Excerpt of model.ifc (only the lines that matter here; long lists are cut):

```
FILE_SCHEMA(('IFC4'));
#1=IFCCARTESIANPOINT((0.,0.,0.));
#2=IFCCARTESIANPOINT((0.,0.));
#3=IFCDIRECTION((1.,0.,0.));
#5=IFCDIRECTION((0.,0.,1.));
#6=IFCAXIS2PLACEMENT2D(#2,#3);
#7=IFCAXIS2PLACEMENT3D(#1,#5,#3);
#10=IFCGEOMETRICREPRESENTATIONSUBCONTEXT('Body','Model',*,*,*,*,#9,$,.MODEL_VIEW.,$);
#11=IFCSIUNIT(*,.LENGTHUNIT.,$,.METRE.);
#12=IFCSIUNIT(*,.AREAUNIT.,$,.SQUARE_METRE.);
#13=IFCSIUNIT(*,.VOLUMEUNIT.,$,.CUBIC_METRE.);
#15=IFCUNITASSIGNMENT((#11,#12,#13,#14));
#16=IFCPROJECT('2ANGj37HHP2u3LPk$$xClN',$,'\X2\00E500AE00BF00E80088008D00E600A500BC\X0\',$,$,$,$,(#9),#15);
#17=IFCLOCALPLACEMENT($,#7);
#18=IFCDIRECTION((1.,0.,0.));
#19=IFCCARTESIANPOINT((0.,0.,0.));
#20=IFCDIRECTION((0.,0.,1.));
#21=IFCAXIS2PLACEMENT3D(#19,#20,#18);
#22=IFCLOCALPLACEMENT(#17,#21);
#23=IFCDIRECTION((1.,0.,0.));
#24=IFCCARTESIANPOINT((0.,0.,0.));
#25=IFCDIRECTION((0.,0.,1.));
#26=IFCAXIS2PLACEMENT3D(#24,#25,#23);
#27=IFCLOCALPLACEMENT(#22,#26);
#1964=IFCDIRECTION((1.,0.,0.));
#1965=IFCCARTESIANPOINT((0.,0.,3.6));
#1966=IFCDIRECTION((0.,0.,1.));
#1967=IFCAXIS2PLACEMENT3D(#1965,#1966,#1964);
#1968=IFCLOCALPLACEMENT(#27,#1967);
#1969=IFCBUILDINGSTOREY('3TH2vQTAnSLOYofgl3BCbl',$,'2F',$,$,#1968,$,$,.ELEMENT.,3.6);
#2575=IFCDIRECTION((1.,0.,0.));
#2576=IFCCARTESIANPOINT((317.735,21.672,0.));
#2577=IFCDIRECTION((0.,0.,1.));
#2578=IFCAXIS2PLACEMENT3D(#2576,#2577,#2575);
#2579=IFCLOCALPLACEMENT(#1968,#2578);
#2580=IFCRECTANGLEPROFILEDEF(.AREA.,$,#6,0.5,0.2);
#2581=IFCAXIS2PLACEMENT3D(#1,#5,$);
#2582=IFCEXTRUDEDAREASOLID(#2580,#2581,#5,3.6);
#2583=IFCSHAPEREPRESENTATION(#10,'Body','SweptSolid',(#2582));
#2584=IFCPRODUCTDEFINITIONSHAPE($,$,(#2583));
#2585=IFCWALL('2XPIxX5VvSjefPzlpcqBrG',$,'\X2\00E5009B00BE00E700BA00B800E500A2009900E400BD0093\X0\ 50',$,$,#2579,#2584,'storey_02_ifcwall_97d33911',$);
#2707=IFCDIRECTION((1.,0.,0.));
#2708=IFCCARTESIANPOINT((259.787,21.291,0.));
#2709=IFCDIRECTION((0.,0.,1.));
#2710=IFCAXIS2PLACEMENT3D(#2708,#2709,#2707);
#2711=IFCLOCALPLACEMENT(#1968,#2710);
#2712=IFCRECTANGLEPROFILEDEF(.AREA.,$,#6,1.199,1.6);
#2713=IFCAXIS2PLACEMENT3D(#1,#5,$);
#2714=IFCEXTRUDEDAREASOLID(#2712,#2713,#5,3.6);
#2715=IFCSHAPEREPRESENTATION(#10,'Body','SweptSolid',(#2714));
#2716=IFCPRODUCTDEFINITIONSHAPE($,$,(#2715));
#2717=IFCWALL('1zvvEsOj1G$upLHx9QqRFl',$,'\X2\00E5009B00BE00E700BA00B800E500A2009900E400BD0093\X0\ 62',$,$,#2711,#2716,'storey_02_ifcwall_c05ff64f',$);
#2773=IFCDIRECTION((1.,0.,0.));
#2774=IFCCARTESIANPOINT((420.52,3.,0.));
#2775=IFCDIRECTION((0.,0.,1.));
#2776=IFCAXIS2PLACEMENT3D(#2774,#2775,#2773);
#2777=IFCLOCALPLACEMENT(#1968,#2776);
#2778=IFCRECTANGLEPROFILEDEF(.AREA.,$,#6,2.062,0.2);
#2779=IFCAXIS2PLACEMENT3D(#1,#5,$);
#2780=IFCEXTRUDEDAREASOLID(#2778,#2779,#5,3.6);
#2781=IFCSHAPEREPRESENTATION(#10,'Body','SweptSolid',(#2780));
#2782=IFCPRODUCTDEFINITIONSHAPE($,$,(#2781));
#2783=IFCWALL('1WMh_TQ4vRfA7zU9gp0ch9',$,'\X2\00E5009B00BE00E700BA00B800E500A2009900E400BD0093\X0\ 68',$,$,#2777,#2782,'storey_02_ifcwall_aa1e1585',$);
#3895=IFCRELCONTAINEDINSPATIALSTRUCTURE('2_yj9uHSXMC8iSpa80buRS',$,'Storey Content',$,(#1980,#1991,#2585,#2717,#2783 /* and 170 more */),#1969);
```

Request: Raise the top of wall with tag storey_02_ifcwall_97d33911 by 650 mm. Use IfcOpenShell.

```python
import ifcopenshell
import ifcopenshell.geom
import ifcopenshell.util.representation
import ifcopenshell.util.shape
import ifcopenshell.util.unit

model = ifcopenshell.open("model.ifc")
unit_scale = ifcopenshell.util.unit.calculate_unit_scale(model)
settings = ifcopenshell.geom.settings()


def volume(element):
    """Net volume in cubic metres, openings subtracted."""
    shape = ifcopenshell.geom.create_shape(settings, element)
    return ifcopenshell.util.shape.get_volume(shape.geometry)


wall = model.by_guid("2XPIxX5VvSjefPzlpcqBrG")
before = volume(wall)

body = ifcopenshell.util.representation.get_representation(wall, "Model", "Body")
solid = body.Items[0]
old_height = solid.Depth
solid.Depth += 0.65 / unit_scale
after = volume(wall)

print(f"height {old_height:g} -> {solid.Depth:g}, volume {before:.3f} -> {after:.3f} m3")

model.write("model_updated.ifc")
```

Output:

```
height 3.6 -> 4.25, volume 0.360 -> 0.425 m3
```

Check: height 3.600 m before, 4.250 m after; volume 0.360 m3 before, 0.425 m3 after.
